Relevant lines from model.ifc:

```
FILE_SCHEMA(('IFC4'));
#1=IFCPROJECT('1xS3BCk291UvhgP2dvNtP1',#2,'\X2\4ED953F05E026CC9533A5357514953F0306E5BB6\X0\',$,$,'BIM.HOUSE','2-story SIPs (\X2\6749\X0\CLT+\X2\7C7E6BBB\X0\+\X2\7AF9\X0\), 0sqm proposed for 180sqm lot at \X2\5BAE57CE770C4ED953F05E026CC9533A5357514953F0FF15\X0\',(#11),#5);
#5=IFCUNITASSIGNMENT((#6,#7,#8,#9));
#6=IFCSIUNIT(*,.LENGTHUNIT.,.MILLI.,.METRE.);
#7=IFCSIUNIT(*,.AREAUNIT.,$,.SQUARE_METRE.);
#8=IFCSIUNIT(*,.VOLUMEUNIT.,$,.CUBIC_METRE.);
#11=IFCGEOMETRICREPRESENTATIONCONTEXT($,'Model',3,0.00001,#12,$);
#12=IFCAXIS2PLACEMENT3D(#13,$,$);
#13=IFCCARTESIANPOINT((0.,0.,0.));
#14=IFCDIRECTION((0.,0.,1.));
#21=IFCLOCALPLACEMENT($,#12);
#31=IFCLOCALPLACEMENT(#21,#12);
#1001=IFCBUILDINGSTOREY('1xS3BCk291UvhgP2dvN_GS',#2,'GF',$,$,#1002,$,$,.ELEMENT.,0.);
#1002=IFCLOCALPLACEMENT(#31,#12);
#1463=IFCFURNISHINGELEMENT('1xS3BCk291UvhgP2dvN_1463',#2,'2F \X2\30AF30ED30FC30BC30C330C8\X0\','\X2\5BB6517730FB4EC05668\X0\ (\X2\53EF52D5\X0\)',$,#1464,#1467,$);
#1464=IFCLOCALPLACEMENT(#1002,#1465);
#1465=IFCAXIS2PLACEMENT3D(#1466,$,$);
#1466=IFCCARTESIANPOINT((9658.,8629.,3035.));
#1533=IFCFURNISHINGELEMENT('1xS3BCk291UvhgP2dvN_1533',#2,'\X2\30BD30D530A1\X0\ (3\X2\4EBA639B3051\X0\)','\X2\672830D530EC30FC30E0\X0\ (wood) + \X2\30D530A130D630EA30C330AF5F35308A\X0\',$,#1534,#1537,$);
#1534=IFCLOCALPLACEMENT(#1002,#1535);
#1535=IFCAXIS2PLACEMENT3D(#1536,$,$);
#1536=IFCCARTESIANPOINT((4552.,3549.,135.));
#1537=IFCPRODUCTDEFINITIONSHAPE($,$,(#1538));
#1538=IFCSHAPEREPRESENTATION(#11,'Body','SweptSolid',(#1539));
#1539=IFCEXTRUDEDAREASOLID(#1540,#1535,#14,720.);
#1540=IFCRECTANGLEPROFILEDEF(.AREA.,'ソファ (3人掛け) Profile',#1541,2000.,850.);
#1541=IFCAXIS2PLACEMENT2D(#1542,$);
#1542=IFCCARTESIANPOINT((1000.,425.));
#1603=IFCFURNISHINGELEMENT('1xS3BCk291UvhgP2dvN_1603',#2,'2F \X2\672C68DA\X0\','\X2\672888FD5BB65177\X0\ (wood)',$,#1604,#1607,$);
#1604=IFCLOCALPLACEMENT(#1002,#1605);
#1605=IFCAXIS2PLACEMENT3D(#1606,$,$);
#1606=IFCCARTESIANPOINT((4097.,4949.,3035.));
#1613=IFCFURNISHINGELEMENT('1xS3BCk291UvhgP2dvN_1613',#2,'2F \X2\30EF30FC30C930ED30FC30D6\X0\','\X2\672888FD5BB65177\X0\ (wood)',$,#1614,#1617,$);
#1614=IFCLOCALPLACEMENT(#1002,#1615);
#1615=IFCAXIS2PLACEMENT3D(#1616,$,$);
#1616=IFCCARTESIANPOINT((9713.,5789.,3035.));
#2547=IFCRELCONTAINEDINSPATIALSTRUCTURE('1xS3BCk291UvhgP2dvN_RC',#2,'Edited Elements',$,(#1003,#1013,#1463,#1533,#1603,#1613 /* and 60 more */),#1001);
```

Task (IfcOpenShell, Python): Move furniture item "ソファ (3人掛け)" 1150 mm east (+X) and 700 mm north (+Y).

```python
import ifcopenshell
import ifcopenshell.api.geometry
import ifcopenshell.util.placement

model = ifcopenshell.open("model.ifc")

item = model.by_guid("1xS3BCk291UvhgP2dvN_1533")
matrix = ifcopenshell.util.placement.get_local_placement(item.ObjectPlacement)
matrix[0, 3] += 1150.0
matrix[1, 3] += 700.0
ifcopenshell.api.geometry.edit_object_placement(model, product=item, matrix=matrix, is_si=False)

print(ifcopenshell.util.placement.get_local_placement(item.ObjectPlacement).round(3) + 0.0)

model.write("model_rev.ifc")
```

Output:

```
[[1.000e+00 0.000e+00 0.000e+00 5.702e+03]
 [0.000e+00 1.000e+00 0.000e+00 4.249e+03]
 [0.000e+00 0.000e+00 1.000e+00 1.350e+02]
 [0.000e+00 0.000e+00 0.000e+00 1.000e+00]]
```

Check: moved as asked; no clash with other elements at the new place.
